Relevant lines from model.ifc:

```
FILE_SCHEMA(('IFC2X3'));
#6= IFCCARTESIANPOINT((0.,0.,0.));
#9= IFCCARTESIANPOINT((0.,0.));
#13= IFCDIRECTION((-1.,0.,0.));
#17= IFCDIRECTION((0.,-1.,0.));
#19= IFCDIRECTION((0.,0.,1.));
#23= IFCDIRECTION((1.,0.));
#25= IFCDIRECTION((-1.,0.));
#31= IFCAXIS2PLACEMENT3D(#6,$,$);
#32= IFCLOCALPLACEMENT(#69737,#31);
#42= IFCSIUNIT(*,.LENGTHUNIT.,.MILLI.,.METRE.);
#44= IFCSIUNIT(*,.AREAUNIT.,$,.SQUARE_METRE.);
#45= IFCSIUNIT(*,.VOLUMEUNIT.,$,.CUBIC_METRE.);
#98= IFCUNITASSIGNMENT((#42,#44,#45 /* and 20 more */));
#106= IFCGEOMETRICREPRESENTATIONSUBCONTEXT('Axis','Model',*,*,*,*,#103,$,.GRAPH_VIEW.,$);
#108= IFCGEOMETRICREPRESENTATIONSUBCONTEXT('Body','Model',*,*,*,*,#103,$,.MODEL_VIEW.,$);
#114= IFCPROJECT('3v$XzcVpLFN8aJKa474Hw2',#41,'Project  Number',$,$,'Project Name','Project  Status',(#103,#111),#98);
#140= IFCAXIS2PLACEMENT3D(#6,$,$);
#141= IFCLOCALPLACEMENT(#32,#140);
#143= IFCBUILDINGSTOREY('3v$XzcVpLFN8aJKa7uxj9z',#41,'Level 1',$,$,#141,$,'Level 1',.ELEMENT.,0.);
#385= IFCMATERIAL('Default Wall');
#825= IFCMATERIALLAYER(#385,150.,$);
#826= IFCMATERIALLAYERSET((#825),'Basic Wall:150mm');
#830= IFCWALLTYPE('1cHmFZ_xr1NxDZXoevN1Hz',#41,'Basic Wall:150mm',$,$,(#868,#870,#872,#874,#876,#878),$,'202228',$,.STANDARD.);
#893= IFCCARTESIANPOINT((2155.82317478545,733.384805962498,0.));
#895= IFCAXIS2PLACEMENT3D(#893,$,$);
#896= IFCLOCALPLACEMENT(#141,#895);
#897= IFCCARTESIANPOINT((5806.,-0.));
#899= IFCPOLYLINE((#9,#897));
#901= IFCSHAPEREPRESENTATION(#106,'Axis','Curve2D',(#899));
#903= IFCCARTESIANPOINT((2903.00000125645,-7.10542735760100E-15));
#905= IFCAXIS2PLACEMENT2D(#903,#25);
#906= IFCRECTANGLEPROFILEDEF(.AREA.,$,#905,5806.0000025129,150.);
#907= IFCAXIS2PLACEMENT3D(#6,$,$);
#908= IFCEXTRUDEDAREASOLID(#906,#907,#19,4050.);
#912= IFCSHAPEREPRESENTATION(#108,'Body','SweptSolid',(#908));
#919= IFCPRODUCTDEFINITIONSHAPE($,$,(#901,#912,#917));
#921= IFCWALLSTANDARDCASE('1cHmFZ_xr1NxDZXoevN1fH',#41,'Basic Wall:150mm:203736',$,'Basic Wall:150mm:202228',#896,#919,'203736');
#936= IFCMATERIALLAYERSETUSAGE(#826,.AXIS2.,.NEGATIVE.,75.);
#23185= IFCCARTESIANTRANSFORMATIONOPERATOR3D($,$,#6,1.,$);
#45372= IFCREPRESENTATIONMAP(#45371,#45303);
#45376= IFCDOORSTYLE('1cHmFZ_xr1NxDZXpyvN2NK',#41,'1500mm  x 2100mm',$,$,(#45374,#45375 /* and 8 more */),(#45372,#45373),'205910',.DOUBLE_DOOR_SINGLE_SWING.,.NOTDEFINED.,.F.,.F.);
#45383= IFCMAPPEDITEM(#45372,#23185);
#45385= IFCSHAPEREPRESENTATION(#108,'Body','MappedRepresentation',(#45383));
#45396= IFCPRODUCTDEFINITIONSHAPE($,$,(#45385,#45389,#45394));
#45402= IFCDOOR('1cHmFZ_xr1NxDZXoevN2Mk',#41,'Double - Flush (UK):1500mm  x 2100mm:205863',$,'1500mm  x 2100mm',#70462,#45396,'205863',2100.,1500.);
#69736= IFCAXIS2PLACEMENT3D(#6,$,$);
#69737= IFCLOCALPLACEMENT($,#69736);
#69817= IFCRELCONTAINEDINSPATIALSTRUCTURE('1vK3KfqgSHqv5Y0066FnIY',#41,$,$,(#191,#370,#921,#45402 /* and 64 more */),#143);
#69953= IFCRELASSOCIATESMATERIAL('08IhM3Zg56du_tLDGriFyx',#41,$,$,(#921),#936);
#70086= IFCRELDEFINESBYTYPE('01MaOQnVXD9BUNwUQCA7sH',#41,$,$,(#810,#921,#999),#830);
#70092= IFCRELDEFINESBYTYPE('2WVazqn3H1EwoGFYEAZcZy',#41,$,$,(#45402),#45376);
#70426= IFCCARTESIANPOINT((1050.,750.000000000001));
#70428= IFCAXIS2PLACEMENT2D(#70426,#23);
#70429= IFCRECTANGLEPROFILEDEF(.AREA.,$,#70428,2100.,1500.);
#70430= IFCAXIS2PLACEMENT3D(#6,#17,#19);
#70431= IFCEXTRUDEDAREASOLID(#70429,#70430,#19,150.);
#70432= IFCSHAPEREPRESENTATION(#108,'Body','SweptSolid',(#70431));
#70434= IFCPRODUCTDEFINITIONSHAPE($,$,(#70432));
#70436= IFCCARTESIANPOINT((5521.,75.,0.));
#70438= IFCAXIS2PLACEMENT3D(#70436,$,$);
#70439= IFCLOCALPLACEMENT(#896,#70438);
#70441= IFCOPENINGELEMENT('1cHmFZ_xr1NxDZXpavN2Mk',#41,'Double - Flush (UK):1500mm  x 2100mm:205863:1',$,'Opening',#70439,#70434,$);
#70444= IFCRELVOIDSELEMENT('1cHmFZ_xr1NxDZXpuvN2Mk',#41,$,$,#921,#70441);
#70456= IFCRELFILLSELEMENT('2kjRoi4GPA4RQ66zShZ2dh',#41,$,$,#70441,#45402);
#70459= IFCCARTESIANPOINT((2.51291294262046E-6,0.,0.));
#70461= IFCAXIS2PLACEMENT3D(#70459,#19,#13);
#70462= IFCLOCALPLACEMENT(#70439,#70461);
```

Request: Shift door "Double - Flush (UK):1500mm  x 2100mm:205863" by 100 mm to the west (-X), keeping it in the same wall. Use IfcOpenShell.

```python
import ifcopenshell
import ifcopenshell.api.geometry
import ifcopenshell.util.placement
import ifcopenshell.util.unit

model = ifcopenshell.open("model.ifc")
unit_scale = ifcopenshell.util.unit.calculate_unit_scale(model)

door = model.by_guid("1cHmFZ_xr1NxDZXoevN2Mk")
opening = door.FillsVoids[0].RelatingOpeningElement
wall = opening.VoidsElements[0].RelatingBuildingElement

wall_matrix = ifcopenshell.util.placement.get_local_placement(wall.ObjectPlacement)
shift = wall_matrix[:3, 0] * -0.1 / unit_scale
before = ifcopenshell.util.placement.get_local_placement(door.ObjectPlacement)[:3, 3].copy()

# The door is placed relative to its opening, so it follows when the opening moves.
matrix = ifcopenshell.util.placement.get_local_placement(opening.ObjectPlacement)
matrix[:3, 3] += shift
ifcopenshell.api.geometry.edit_object_placement(
    model, product=opening, matrix=matrix, is_si=False, should_transform_children=True
)

after = ifcopenshell.util.placement.get_local_placement(door.ObjectPlacement)[:3, 3]
print("door moved by", (after - before).round(3) + 0.0)

model.write("model_edited.ifc")
```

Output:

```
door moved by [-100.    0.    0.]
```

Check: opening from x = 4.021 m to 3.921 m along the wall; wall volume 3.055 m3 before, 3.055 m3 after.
